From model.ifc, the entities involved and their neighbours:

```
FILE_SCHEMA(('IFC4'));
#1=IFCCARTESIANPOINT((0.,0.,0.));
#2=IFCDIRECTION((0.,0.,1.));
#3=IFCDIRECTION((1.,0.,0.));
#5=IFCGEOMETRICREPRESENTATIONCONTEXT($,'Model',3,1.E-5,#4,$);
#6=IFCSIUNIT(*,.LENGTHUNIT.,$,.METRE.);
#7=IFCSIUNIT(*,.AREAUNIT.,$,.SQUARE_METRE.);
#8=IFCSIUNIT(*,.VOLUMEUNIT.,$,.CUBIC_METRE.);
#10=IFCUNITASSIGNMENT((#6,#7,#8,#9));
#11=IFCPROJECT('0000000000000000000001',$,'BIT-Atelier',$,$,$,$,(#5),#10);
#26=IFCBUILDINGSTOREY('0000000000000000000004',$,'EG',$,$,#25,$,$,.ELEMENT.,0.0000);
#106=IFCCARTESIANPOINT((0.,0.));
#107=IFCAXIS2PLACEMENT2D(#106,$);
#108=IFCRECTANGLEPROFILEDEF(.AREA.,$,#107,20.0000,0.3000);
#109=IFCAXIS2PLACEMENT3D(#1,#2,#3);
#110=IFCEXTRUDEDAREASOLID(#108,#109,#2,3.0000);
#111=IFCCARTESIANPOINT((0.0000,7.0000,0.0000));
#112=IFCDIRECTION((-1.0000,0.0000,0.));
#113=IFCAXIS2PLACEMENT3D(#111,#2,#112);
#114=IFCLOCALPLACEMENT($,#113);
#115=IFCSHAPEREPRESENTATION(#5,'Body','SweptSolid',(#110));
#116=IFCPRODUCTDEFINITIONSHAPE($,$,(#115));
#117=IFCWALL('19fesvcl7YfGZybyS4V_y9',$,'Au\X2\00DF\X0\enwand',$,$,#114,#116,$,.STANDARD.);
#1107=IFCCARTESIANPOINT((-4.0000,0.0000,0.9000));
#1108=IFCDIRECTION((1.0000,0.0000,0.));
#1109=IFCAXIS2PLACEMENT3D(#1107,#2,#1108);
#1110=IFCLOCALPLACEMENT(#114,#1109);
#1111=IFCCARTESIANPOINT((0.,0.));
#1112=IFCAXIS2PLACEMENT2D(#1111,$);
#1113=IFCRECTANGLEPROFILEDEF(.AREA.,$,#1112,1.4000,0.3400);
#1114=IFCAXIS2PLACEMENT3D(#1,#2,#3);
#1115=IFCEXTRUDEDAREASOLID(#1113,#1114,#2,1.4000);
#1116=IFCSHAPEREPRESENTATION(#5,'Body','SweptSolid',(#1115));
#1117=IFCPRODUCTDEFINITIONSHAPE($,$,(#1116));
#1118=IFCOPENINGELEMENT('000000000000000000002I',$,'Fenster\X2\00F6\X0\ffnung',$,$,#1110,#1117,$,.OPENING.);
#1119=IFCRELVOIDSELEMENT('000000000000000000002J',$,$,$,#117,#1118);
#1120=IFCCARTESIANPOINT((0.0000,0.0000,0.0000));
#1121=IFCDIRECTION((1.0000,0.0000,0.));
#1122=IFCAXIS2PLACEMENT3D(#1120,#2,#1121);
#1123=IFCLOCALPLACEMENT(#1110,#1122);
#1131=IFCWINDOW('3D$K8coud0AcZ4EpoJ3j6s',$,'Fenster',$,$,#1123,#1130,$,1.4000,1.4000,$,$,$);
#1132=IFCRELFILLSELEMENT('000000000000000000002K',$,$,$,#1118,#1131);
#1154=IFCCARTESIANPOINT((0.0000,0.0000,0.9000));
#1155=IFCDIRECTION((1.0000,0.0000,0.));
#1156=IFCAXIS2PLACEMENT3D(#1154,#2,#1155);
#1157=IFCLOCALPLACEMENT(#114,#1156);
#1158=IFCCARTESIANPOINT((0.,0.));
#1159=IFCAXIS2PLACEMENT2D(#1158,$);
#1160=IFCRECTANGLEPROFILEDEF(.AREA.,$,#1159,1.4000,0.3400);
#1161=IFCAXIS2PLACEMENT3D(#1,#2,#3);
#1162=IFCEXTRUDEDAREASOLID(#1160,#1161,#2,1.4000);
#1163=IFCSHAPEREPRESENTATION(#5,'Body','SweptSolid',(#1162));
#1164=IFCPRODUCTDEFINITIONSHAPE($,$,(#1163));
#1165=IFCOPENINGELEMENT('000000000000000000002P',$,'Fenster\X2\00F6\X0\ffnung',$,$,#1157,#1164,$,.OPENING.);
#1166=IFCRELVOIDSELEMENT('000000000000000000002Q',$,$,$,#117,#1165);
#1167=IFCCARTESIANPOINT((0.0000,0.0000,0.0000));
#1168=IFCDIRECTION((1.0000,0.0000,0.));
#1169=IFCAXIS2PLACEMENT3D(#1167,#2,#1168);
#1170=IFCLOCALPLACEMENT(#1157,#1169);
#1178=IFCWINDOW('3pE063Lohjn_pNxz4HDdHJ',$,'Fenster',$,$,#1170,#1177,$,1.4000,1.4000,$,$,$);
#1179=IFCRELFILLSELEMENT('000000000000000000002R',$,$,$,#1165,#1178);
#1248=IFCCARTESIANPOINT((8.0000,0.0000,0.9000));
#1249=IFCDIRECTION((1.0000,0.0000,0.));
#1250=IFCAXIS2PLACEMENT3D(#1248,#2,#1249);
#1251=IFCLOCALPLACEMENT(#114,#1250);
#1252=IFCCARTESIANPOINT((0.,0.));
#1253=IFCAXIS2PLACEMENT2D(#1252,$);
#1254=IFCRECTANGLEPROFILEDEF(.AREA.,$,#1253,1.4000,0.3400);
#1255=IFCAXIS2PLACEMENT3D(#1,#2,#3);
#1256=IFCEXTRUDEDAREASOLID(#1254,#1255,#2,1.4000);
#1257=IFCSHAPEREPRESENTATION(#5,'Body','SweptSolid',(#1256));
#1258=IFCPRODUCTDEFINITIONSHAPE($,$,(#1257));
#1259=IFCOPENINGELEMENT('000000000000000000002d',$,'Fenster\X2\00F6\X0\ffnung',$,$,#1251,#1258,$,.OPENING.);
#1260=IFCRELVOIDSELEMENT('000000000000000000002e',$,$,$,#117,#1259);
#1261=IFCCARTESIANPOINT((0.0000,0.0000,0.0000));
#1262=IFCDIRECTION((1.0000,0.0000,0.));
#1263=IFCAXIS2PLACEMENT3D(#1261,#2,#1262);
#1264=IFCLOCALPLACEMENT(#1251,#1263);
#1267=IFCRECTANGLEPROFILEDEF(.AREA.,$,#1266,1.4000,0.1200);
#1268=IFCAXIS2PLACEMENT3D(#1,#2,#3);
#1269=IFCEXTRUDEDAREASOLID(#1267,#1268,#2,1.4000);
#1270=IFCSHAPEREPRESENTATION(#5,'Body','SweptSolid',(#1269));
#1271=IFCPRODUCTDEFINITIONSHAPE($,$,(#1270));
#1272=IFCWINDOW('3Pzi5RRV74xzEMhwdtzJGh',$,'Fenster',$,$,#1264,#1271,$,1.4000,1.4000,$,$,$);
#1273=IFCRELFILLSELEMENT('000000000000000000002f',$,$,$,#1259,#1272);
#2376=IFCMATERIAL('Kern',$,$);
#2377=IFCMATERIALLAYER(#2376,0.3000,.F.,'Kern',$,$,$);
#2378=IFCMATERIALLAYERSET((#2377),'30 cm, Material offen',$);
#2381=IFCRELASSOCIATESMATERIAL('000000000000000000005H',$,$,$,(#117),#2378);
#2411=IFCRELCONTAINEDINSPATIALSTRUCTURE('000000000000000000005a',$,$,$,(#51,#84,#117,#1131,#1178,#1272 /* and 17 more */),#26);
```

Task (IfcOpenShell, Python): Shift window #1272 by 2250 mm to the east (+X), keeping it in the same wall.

```python
import ifcopenshell
import ifcopenshell.api.geometry
import ifcopenshell.util.placement

model = ifcopenshell.open("model.ifc")

window = model.by_guid("3Pzi5RRV74xzEMhwdtzJGh")
opening = window.FillsVoids[0].RelatingOpeningElement
wall = opening.VoidsElements[0].RelatingBuildingElement

wall_matrix = ifcopenshell.util.placement.get_local_placement(wall.ObjectPlacement)
shift = wall_matrix[:3, 0] * -2.25
before = ifcopenshell.util.placement.get_local_placement(window.ObjectPlacement)[:3, 3].copy()

# The window is placed relative to its opening, so it follows when the opening moves.
matrix = ifcopenshell.util.placement.get_local_placement(opening.ObjectPlacement)
matrix[:3, 3] += shift
ifcopenshell.api.geometry.edit_object_placement(
    model, product=opening, matrix=matrix, is_si=False, should_transform_children=True
)

after = ifcopenshell.util.placement.get_local_placement(window.ObjectPlacement)[:3, 3]
print("window moved by", (after - before).round(3) + 0.0)

model.write("model_rev.ifc")
```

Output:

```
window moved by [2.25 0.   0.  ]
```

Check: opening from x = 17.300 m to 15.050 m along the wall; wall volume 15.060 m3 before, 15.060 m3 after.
